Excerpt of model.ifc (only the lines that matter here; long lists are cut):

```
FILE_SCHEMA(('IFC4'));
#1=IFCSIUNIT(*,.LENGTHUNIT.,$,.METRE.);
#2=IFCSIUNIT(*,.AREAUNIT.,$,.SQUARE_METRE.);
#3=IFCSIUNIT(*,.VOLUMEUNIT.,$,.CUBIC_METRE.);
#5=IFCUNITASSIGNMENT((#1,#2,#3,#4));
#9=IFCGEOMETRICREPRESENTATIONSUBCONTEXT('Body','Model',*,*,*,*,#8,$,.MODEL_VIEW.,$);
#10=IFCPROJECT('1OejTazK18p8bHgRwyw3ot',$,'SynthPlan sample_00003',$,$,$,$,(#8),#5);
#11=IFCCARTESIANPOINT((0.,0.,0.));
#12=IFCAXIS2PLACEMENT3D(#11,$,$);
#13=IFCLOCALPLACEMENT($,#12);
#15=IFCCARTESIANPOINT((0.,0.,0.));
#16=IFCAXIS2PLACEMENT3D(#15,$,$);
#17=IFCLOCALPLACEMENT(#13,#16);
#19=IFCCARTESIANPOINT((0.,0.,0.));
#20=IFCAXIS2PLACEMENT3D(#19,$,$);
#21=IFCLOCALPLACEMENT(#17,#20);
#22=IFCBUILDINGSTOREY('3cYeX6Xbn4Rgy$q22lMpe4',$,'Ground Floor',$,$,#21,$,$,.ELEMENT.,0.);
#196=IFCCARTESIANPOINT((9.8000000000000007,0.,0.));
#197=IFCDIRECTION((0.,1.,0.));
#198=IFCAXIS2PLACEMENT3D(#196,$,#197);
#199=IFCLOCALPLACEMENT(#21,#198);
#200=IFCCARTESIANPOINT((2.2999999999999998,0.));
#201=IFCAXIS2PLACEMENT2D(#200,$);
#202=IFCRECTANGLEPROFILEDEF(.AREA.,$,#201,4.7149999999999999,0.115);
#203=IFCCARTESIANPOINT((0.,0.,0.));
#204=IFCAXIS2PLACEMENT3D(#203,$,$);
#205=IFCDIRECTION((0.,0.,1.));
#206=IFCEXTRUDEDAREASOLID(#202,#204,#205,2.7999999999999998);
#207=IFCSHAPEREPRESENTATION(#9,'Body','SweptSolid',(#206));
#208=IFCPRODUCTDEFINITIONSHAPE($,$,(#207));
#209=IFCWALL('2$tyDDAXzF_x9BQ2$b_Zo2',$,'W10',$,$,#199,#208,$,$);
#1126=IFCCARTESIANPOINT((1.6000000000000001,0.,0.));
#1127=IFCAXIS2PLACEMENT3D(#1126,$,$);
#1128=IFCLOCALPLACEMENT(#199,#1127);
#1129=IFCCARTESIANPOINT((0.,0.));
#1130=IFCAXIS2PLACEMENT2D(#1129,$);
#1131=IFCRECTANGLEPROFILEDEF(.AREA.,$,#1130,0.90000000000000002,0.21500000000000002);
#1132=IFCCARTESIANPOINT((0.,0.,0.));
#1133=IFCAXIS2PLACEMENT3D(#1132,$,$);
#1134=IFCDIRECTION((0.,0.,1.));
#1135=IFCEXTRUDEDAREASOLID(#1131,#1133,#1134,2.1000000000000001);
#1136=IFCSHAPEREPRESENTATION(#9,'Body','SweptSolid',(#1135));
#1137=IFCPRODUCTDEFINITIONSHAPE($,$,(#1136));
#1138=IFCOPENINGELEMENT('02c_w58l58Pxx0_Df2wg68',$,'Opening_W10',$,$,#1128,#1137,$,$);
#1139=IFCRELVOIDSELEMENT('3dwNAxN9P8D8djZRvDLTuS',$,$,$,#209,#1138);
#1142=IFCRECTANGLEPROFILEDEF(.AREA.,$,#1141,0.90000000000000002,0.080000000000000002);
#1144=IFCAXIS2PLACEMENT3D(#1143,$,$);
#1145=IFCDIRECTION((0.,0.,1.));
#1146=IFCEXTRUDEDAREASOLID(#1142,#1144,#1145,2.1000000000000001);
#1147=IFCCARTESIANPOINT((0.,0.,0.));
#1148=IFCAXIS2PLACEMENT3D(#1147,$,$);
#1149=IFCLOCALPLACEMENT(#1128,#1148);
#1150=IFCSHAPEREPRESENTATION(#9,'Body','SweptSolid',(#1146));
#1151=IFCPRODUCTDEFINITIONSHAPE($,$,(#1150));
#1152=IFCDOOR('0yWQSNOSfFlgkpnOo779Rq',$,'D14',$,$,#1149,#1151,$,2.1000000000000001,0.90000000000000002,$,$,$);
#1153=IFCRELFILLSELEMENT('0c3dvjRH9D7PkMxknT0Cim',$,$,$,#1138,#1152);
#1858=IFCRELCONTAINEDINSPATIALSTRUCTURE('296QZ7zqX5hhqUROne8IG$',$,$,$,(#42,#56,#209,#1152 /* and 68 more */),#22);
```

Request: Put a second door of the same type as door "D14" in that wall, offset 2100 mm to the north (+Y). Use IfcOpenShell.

```python
import ifcopenshell
import ifcopenshell.api.feature
import ifcopenshell.api.geometry
import ifcopenshell.api.root
import ifcopenshell.geom
import ifcopenshell.util.element
import ifcopenshell.util.placement
import ifcopenshell.util.shape

model = ifcopenshell.open("model.ifc")
settings = ifcopenshell.geom.settings()


def volume(element):
    """Net volume in cubic metres, openings subtracted."""
    shape = ifcopenshell.geom.create_shape(settings, element)
    return ifcopenshell.util.shape.get_volume(shape.geometry)


door = model.by_guid("0yWQSNOSfFlgkpnOo779Rq")
opening = door.FillsVoids[0].RelatingOpeningElement
wall = opening.VoidsElements[0].RelatingBuildingElement
before = volume(wall)
shift = ifcopenshell.util.placement.get_local_placement(wall.ObjectPlacement)[:3, 0] * 2.1

# copy_class copies the void relationship, type, container and properties, but no geometry.
new_opening = ifcopenshell.api.root.copy_class(model, product=opening)
new_opening.Representation = ifcopenshell.util.element.copy_deep(
    model, opening.Representation, exclude=["IfcGeometricRepresentationContext", "IfcRepresentationMap"]
)
new_door = ifcopenshell.api.root.copy_class(model, product=door)
new_door.Representation = ifcopenshell.util.element.copy_deep(
    model, door.Representation, exclude=["IfcGeometricRepresentationContext", "IfcRepresentationMap"]
)
ifcopenshell.api.feature.add_filling(model, opening=new_opening, element=new_door)

for old, new in ((opening, new_opening), (door, new_door)):
    matrix = ifcopenshell.util.placement.get_local_placement(old.ObjectPlacement)
    matrix[:3, 3] += shift
    ifcopenshell.api.geometry.edit_object_placement(model, product=new, matrix=matrix, is_si=False)

after = volume(wall)

print(f"wall volume {before:.3f} -> {after:.3f} m3")

model.write("model_edited.ifc")
```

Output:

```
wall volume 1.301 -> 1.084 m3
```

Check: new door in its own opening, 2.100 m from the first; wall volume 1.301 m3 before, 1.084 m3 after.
